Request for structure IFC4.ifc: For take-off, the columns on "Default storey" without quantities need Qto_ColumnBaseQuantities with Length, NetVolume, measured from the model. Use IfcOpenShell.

First a look at what the model holds.

```python
import ifcopenshell
import ifcopenshell.util.element
import ifcopenshell.util.unit

model = ifcopenshell.open("structure IFC4.ifc")
print(model.schema)
for unit_type in ("LENGTHUNIT", "AREAUNIT", "VOLUMEUNIT"):
    print(unit_type, ifcopenshell.util.unit.calculate_unit_scale(model, unit_type))
storey = next(s for s in model.by_type("IfcBuildingStorey") if s.Name == "Default storey")
columns = [e for e in ifcopenshell.util.element.get_decomposition(storey) if e.is_a("IfcColumn")]
for e in sorted(columns, key=lambda e: e.id()):
    print(e.id(), e.is_a(), e.Name, list(ifcopenshell.util.element.get_psets(e, qtos_only=True)), sep=" | ")
```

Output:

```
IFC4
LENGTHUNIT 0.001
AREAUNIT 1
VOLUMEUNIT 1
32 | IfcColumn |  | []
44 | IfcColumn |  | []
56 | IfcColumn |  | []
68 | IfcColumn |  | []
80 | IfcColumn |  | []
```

```python
import ifcopenshell
import ifcopenshell.api.pset
import ifcopenshell.geom
import ifcopenshell.util.element
import ifcopenshell.util.shape
import ifcopenshell.util.unit

model = ifcopenshell.open("structure IFC4.ifc")
unit_scale = ifcopenshell.util.unit.calculate_unit_scale(model)
volume_scale = ifcopenshell.util.unit.calculate_unit_scale(model, "VOLUMEUNIT")
settings = ifcopenshell.geom.settings()

storey = next(s for s in model.by_type("IfcBuildingStorey") if s.Name == "Default storey")
columns = [e for e in ifcopenshell.util.element.get_decomposition(storey) if e.is_a("IfcColumn")]

for e in sorted(columns, key=lambda e: e.id()):
    if ifcopenshell.util.element.get_psets(e, qtos_only=True, should_inherit=False):
        continue
    # Geometry comes back in metres, in the element's own axes.
    shape = ifcopenshell.geom.create_shape(settings, e)
    values = {
        "Length": ifcopenshell.util.shape.get_z(shape.geometry) / unit_scale,
        "NetVolume": ifcopenshell.util.shape.get_volume(shape.geometry) / volume_scale,
    }
    qto = ifcopenshell.api.pset.add_qto(model, product=e, name="Qto_ColumnBaseQuantities")
    ifcopenshell.api.pset.edit_qto(model, qto=qto, properties=values)
    print(e.id(), {k: round(v, 3) for k, v in values.items()})

model.write("structure IFC4_edited.ifc")
```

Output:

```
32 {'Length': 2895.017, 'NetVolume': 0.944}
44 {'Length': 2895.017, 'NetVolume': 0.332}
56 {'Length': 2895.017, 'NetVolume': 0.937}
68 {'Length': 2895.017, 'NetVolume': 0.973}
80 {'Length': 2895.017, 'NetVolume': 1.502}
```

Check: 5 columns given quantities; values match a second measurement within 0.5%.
